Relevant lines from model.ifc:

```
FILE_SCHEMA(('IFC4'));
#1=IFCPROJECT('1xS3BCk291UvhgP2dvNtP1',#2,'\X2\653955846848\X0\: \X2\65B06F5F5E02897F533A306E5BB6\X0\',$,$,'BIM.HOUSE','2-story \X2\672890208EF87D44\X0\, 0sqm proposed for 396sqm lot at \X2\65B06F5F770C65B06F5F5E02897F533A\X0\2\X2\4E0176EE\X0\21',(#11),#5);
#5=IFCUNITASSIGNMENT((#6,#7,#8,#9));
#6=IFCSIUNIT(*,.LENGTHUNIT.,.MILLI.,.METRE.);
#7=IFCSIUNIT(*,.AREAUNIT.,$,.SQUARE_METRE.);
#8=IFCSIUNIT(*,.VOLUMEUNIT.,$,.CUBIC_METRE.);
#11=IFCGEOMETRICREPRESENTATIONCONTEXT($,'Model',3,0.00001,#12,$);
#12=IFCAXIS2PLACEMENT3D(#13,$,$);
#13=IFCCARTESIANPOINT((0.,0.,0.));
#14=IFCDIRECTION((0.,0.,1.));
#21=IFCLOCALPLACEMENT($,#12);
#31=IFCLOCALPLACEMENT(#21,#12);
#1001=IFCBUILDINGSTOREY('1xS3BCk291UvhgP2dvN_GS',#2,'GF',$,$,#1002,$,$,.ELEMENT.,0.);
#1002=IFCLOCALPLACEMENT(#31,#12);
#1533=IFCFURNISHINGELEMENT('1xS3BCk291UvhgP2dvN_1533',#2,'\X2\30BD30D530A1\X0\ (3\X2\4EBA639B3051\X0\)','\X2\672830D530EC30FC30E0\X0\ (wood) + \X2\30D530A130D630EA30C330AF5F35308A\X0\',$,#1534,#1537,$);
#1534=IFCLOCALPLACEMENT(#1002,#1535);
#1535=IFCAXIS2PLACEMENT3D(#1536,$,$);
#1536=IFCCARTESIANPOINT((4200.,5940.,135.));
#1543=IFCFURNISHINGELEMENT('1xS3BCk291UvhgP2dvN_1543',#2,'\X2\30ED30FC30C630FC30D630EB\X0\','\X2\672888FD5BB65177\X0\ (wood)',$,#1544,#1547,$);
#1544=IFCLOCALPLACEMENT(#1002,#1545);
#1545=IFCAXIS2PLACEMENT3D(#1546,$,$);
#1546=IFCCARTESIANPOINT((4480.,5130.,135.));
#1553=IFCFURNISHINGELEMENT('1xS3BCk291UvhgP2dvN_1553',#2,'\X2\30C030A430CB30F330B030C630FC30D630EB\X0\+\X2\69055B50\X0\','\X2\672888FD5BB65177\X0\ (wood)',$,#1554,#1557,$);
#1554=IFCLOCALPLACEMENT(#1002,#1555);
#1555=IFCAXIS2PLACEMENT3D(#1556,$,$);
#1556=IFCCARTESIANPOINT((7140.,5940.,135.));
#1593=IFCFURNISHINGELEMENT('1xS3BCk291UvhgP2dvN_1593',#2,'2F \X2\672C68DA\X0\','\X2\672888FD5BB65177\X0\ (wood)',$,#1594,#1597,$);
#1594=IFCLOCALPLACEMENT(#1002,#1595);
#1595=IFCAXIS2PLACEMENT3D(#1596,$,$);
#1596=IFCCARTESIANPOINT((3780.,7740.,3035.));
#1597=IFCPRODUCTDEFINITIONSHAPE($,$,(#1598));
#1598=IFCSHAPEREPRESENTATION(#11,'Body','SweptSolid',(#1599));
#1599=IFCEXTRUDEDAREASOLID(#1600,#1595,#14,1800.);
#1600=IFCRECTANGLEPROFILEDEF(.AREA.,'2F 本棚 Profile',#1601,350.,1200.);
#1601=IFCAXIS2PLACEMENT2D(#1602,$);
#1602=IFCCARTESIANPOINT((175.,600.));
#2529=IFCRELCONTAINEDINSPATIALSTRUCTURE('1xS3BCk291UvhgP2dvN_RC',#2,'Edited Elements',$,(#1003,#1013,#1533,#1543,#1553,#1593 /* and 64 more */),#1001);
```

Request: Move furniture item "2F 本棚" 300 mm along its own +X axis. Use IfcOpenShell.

```python
import ifcopenshell
import ifcopenshell.api.geometry
import ifcopenshell.util.placement
import ifcopenshell.util.unit

model = ifcopenshell.open("model.ifc")
unit_scale = ifcopenshell.util.unit.calculate_unit_scale(model)

item = model.by_guid("1xS3BCk291UvhgP2dvN_1593")
matrix = ifcopenshell.util.placement.get_local_placement(item.ObjectPlacement)
matrix[:3, 3] += matrix[:3, 0] * 0.3 / unit_scale
ifcopenshell.api.geometry.edit_object_placement(model, product=item, matrix=matrix, is_si=False)

print(ifcopenshell.util.placement.get_local_placement(item.ObjectPlacement).round(3) + 0.0)

model.write("model-out.ifc")
```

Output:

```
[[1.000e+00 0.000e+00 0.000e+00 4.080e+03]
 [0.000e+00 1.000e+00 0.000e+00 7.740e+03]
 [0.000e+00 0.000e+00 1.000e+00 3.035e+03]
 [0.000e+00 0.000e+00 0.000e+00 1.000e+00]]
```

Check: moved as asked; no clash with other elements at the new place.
